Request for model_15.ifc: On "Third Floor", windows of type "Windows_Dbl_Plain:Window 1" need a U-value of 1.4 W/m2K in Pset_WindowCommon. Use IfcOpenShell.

First a look at what the model holds.

```python
import ifcopenshell
import ifcopenshell.util.element

model = ifcopenshell.open("model_15.ifc")
print(model.schema)
storey = next(s for s in model.by_type("IfcBuildingStorey") if s.Name == "Third Floor")
windows = [e for e in ifcopenshell.util.element.get_decomposition(storey) if e.is_a("IfcWindow")]
seen = {}
for e in windows:
    element_type = ifcopenshell.util.element.get_type(e)
    key = (element_type.Name if element_type != e and element_type else None, ifcopenshell.util.element.get_pset(e, "Pset_WindowCommon", "ThermalTransmittance"))
    seen[key] = seen.get(key, 0) + 1
for (name, value), count in sorted(seen.items(), key=str):
    print(count, "x", name, "|", value)
```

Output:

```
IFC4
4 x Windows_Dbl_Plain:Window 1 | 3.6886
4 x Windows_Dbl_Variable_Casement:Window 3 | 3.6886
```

```python
import ifcopenshell
import ifcopenshell.api.pset
import ifcopenshell.util.element

model = ifcopenshell.open("model_15.ifc")

storey = next(s for s in model.by_type("IfcBuildingStorey") if s.Name == "Third Floor")
windows = [e for e in ifcopenshell.util.element.get_decomposition(storey) if e.is_a("IfcWindow")]

count = 0
for e in windows:
    element_type = ifcopenshell.util.element.get_type(e)
    if element_type in (None, e) or element_type.Name != "Windows_Dbl_Plain:Window 1":
        continue
    # add_pset returns the element's existing set when there is one.
    pset = ifcopenshell.api.pset.add_pset(model, product=e, name="Pset_WindowCommon")
    ifcopenshell.api.pset.edit_pset(model, pset=pset, properties={"ThermalTransmittance": 1.4})
    count += 1

print(count, "windows updated")

model.write("model_15-out.ifc")
```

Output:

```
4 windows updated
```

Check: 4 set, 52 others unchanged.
